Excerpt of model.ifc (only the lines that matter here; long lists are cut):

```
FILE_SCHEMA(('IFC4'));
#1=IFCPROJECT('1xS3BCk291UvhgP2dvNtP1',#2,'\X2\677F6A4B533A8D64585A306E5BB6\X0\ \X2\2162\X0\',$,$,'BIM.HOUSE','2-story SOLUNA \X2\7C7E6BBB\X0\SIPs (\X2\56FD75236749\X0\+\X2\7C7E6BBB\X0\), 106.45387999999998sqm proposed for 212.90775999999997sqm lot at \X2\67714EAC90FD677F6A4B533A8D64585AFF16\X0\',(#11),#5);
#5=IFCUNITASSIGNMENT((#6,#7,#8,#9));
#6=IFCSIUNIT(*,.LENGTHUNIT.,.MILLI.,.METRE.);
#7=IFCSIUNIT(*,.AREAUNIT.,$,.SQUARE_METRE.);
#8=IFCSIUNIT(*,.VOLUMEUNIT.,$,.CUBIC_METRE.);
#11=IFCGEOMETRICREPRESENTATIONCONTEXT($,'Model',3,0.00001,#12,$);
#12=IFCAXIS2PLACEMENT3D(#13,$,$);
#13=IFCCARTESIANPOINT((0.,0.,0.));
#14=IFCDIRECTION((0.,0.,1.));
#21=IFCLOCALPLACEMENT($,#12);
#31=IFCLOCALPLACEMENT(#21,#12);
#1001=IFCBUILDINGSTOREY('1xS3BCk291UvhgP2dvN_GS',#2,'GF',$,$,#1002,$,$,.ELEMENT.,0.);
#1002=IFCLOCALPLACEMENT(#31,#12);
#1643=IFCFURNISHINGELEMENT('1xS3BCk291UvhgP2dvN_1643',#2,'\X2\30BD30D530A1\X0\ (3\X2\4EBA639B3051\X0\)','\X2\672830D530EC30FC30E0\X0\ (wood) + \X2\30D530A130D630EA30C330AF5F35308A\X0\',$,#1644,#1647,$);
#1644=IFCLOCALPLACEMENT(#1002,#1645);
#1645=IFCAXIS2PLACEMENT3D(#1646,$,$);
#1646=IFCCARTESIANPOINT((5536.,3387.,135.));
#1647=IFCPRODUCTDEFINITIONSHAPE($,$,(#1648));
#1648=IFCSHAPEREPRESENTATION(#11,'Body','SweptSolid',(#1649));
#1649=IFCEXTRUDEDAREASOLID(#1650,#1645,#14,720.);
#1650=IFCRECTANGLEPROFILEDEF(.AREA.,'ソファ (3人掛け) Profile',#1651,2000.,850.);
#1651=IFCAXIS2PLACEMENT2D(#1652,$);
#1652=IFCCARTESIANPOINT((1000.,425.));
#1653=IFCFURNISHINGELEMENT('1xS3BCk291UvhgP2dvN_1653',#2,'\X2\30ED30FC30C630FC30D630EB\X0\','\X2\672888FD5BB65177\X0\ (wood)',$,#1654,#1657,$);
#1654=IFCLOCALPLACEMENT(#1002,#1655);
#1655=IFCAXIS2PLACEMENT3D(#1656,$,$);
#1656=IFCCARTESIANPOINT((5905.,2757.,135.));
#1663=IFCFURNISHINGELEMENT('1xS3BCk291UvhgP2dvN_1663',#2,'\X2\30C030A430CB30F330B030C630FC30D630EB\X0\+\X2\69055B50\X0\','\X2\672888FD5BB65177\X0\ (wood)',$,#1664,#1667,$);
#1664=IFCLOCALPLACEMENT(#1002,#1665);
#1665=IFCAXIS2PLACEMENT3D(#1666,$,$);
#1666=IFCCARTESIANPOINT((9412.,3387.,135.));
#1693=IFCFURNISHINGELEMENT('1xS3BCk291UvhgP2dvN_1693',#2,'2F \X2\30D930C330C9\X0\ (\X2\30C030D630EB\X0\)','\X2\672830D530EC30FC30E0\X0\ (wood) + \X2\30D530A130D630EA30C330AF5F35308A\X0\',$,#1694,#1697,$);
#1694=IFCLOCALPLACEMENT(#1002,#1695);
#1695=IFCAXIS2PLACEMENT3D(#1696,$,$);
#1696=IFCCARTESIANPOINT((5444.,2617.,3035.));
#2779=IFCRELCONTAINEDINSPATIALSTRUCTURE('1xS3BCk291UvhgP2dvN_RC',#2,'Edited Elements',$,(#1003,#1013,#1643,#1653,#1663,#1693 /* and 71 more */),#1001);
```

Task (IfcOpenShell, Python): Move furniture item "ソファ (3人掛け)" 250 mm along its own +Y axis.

```python
import ifcopenshell
import ifcopenshell.api.geometry
import ifcopenshell.util.placement
import ifcopenshell.util.unit

model = ifcopenshell.open("model.ifc")
unit_scale = ifcopenshell.util.unit.calculate_unit_scale(model)

item = model.by_guid("1xS3BCk291UvhgP2dvN_1643")
matrix = ifcopenshell.util.placement.get_local_placement(item.ObjectPlacement)
matrix[:3, 3] += matrix[:3, 1] * 0.25 / unit_scale
ifcopenshell.api.geometry.edit_object_placement(model, product=item, matrix=matrix, is_si=False)

print(ifcopenshell.util.placement.get_local_placement(item.ObjectPlacement).round(3) + 0.0)

model.write("model_edited.ifc")
```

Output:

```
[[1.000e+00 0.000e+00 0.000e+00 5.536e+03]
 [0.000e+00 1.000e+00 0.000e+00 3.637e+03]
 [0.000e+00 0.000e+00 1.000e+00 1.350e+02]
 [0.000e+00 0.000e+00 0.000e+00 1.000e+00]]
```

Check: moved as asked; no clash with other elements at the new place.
